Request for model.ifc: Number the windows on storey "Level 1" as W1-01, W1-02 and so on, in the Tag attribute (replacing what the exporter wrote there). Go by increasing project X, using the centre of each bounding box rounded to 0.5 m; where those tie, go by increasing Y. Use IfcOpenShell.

First a look at what the model holds.

```python
import ifcopenshell
import ifcopenshell.util.element
import ifcopenshell.util.placement

model = ifcopenshell.open("model.ifc")
print(model.schema)
storey = next(s for s in model.by_type("IfcBuildingStorey") if s.Name == "Level 1")
windows = [e for e in ifcopenshell.util.element.get_decomposition(storey) if e.is_a("IfcWindow")]
for e in sorted(windows, key=lambda e: e.id()):
    origin = ifcopenshell.util.placement.get_local_placement(e.ObjectPlacement)[:3, 3]
    print(e.id(), e.Tag, e.Name, origin.round(2) + 0.0, sep=" | ")
```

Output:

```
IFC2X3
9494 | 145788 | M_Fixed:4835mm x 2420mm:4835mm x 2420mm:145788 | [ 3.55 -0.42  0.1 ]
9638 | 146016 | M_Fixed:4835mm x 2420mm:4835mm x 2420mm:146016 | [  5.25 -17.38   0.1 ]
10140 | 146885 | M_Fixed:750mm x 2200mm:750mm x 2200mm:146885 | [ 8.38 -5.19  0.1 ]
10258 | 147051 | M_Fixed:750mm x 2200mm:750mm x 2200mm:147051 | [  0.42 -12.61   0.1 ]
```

```python
import ifcopenshell
import ifcopenshell.geom
import ifcopenshell.util.element
import ifcopenshell.util.shape

model = ifcopenshell.open("model.ifc")
settings = ifcopenshell.geom.settings()
settings.set("use-world-coords", True)


def centre(element):
    shape = ifcopenshell.geom.create_shape(settings, element)
    return ifcopenshell.util.shape.get_bbox_centroid(shape.geometry)


storey = next(s for s in model.by_type("IfcBuildingStorey") if s.Name == "Level 1")
windows = [e for e in ifcopenshell.util.element.get_decomposition(storey) if e.is_a("IfcWindow")]

# Insertion points can sit at a corner or the storey origin, so sort by the geometry (in metres).
centres = {e: centre(e) for e in windows}
windows.sort(key=lambda e: (round(centres[e][0] / 0.5), centres[e][1]))

for i, e in enumerate(windows, start=1):
    number = f"W1-{i:02d}"
    e.Tag = number
    print(e.id(), number)

model.write("model_edited.ifc")
```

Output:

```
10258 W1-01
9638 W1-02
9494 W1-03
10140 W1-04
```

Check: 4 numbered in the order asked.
